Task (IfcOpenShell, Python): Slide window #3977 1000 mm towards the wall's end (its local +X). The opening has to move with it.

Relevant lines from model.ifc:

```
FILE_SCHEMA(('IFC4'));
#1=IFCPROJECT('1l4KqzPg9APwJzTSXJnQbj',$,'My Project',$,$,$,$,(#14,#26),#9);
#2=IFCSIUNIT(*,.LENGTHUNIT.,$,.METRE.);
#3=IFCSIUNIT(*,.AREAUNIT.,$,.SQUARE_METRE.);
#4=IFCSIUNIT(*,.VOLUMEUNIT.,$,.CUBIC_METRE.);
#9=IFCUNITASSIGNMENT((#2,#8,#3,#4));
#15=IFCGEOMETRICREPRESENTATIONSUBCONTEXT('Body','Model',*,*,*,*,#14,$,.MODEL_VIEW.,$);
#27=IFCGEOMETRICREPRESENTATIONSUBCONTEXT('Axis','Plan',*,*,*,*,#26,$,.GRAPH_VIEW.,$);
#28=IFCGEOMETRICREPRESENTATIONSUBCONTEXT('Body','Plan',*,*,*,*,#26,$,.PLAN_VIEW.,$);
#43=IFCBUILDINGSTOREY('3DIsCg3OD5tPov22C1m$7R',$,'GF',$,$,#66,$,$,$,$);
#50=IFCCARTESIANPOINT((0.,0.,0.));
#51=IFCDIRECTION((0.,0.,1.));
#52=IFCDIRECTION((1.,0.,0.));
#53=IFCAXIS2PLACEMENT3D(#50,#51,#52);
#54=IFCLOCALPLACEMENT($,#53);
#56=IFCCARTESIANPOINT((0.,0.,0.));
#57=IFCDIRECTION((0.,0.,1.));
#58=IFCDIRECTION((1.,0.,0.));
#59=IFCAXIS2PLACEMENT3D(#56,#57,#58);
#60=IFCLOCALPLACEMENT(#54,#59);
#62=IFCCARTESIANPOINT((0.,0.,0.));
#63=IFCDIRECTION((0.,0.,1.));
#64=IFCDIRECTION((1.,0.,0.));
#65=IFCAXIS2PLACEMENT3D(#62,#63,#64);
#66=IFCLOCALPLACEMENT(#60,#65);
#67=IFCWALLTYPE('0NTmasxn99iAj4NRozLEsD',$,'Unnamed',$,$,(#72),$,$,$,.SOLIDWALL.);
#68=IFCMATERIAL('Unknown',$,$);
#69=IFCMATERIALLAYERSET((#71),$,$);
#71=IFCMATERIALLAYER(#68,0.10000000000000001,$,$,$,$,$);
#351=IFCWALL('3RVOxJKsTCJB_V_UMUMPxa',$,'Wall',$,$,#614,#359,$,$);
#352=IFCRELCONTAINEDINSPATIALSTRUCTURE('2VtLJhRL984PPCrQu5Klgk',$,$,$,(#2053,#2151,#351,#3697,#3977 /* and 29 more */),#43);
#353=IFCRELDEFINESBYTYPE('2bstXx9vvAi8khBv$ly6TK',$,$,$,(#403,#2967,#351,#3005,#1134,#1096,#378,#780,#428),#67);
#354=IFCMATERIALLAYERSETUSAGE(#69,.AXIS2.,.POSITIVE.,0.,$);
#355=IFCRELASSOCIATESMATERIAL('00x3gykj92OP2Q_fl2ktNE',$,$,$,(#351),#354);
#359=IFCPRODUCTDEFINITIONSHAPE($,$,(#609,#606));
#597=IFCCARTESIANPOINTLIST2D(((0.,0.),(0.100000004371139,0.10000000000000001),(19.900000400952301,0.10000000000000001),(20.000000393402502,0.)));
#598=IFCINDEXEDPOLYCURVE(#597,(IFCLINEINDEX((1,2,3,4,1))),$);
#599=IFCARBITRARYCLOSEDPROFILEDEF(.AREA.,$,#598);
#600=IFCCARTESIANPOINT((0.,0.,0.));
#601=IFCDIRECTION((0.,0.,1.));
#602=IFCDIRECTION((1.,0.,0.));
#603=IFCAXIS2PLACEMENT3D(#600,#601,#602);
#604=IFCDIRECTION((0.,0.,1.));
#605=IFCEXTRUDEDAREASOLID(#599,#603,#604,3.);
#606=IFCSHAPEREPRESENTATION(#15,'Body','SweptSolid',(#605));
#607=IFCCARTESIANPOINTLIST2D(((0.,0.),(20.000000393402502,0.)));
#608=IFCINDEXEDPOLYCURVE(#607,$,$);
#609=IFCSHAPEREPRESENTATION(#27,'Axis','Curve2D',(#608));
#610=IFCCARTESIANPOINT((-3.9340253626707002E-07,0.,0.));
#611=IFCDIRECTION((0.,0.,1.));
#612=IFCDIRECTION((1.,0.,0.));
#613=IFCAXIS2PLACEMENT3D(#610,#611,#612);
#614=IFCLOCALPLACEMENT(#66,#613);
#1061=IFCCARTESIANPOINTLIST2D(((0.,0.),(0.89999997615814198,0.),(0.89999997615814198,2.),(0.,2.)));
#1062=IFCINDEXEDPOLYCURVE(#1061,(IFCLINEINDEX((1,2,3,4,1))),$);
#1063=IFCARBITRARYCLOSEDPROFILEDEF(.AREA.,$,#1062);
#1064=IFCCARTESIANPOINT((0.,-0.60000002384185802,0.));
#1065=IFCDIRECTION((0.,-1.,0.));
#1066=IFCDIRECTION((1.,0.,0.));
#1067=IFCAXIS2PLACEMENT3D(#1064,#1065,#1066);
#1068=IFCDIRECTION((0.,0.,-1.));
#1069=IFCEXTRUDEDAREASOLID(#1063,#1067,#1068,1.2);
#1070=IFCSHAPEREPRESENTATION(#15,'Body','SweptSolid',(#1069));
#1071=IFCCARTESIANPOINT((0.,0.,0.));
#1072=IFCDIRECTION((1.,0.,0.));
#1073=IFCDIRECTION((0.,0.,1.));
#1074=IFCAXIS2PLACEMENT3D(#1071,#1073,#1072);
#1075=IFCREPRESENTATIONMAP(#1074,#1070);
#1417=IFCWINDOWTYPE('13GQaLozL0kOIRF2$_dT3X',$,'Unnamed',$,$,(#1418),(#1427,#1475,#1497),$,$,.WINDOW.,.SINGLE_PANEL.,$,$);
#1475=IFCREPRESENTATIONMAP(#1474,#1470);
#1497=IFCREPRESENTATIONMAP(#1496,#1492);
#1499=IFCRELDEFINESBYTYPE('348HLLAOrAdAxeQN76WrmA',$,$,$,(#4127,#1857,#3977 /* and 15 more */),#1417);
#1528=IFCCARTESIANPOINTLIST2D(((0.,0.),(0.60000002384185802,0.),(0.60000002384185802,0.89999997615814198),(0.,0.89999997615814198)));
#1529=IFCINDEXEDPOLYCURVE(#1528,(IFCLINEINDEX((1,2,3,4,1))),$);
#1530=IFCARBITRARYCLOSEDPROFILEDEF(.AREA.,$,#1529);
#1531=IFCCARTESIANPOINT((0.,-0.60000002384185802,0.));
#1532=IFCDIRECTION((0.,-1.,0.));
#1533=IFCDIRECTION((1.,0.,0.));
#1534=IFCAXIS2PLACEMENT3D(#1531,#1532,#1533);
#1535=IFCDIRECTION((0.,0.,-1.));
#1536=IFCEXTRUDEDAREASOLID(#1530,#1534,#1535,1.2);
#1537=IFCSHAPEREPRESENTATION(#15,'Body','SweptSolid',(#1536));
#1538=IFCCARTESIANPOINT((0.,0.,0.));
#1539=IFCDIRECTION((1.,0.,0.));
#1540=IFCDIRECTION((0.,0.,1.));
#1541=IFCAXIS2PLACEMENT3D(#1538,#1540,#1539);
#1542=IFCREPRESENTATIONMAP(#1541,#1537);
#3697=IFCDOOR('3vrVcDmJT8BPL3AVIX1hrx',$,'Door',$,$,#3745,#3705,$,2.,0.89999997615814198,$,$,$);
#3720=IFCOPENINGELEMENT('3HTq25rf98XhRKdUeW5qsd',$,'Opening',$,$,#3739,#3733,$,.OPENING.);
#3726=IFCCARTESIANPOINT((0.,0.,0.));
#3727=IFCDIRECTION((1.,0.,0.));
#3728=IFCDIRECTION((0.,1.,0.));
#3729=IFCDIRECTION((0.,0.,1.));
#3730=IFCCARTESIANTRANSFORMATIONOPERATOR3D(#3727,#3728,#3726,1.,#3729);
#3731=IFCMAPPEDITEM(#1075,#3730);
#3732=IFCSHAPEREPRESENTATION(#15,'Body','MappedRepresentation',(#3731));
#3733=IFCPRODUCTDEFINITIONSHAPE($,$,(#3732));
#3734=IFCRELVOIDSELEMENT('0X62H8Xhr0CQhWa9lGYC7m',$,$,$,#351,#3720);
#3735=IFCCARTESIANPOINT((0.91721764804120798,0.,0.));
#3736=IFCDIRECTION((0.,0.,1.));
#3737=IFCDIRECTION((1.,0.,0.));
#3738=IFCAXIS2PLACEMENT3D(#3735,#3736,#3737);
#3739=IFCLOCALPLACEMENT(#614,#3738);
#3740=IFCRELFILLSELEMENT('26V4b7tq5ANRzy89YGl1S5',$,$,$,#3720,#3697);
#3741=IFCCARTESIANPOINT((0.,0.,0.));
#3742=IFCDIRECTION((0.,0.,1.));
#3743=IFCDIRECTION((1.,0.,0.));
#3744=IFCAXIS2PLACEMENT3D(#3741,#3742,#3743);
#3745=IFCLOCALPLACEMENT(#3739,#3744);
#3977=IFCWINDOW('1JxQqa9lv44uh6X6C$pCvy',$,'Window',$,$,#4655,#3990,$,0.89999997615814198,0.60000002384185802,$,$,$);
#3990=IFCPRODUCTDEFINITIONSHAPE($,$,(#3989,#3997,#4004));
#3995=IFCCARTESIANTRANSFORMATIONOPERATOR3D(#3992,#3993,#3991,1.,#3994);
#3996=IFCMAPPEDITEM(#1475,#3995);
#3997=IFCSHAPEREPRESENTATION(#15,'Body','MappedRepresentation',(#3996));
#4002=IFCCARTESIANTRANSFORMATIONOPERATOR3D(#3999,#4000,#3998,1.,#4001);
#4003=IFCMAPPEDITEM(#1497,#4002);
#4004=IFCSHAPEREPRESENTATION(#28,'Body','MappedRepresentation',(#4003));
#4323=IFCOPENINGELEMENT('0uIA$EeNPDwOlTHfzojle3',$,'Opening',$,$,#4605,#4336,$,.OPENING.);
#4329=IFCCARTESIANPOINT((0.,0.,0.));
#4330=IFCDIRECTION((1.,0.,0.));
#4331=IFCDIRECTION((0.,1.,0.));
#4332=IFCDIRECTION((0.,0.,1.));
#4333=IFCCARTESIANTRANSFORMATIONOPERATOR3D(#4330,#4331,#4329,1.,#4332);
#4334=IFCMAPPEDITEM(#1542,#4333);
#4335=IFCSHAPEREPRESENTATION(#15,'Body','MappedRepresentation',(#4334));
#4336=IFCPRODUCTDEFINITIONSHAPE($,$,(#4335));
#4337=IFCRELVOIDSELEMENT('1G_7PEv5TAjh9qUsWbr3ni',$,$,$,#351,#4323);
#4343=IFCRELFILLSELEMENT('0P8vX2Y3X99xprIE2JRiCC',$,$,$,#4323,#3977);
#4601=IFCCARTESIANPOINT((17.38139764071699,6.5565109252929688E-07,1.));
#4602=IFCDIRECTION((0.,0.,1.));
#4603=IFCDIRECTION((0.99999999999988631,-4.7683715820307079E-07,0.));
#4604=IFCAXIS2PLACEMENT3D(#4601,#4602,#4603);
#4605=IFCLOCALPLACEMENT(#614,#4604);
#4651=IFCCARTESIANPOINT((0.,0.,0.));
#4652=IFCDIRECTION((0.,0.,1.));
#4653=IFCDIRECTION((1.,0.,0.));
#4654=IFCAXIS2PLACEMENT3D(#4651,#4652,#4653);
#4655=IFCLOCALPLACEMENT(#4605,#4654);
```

```python
import ifcopenshell
import ifcopenshell.api.geometry
import ifcopenshell.util.placement
import ifcopenshell.util.unit

model = ifcopenshell.open("model.ifc")
unit_scale = ifcopenshell.util.unit.calculate_unit_scale(model)

window = model.by_id(3977)
opening = window.FillsVoids[0].RelatingOpeningElement
wall = opening.VoidsElements[0].RelatingBuildingElement

wall_matrix = ifcopenshell.util.placement.get_local_placement(wall.ObjectPlacement)
shift = wall_matrix[:3, 0] * 1 / unit_scale
before = ifcopenshell.util.placement.get_local_placement(window.ObjectPlacement)[:3, 3].copy()

# The window is placed relative to its opening, so it follows when the opening moves.
matrix = ifcopenshell.util.placement.get_local_placement(opening.ObjectPlacement)
matrix[:3, 3] += shift
ifcopenshell.api.geometry.edit_object_placement(
    model, product=opening, matrix=matrix, is_si=False, should_transform_children=True
)

after = ifcopenshell.util.placement.get_local_placement(window.ObjectPlacement)[:3, 3]
print("window moved by", (after - before).round(3) + 0.0)

model.write("model_edited.ifc")
```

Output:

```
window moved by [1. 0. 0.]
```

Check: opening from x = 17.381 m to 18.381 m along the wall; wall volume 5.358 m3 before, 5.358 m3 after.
